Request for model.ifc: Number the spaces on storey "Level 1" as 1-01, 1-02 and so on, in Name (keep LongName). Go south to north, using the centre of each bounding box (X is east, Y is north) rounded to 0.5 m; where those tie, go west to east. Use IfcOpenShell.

First a look at what the model holds.

```python
import ifcopenshell
import ifcopenshell.util.element
import ifcopenshell.util.placement

model = ifcopenshell.open("model.ifc")
print(model.schema)
storey = next(s for s in model.by_type("IfcBuildingStorey") if s.Name == "Level 1")
spaces = [e for e in ifcopenshell.util.element.get_decomposition(storey) if e.is_a("IfcSpace")]
for e in sorted(spaces, key=lambda e: e.id()):
    origin = ifcopenshell.util.placement.get_local_placement(e.ObjectPlacement)[:3, 3]
    print(e.id(), e.Name, e.LongName, origin.round(2) + 0.0, sep=" | ")
```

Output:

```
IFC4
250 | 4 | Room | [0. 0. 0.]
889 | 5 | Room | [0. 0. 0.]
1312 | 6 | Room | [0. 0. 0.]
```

```python
import ifcopenshell
import ifcopenshell.geom
import ifcopenshell.util.element
import ifcopenshell.util.shape

model = ifcopenshell.open("model.ifc")
settings = ifcopenshell.geom.settings()
settings.set("use-world-coords", True)


def centre(element):
    shape = ifcopenshell.geom.create_shape(settings, element)
    return ifcopenshell.util.shape.get_bbox_centroid(shape.geometry)


storey = next(s for s in model.by_type("IfcBuildingStorey") if s.Name == "Level 1")
spaces = [e for e in ifcopenshell.util.element.get_decomposition(storey) if e.is_a("IfcSpace")]

# Insertion points can sit at a corner or the storey origin, so sort by the geometry (in metres).
centres = {e: centre(e) for e in spaces}
spaces.sort(key=lambda e: (round(centres[e][1] / 0.5), centres[e][0]))

for i, e in enumerate(spaces, start=1):
    number = f"1-{i:02d}"
    e.Name = number
    print(e.id(), number)

model.write("model_rev.ifc")
```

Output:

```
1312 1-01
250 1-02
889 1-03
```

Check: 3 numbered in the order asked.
